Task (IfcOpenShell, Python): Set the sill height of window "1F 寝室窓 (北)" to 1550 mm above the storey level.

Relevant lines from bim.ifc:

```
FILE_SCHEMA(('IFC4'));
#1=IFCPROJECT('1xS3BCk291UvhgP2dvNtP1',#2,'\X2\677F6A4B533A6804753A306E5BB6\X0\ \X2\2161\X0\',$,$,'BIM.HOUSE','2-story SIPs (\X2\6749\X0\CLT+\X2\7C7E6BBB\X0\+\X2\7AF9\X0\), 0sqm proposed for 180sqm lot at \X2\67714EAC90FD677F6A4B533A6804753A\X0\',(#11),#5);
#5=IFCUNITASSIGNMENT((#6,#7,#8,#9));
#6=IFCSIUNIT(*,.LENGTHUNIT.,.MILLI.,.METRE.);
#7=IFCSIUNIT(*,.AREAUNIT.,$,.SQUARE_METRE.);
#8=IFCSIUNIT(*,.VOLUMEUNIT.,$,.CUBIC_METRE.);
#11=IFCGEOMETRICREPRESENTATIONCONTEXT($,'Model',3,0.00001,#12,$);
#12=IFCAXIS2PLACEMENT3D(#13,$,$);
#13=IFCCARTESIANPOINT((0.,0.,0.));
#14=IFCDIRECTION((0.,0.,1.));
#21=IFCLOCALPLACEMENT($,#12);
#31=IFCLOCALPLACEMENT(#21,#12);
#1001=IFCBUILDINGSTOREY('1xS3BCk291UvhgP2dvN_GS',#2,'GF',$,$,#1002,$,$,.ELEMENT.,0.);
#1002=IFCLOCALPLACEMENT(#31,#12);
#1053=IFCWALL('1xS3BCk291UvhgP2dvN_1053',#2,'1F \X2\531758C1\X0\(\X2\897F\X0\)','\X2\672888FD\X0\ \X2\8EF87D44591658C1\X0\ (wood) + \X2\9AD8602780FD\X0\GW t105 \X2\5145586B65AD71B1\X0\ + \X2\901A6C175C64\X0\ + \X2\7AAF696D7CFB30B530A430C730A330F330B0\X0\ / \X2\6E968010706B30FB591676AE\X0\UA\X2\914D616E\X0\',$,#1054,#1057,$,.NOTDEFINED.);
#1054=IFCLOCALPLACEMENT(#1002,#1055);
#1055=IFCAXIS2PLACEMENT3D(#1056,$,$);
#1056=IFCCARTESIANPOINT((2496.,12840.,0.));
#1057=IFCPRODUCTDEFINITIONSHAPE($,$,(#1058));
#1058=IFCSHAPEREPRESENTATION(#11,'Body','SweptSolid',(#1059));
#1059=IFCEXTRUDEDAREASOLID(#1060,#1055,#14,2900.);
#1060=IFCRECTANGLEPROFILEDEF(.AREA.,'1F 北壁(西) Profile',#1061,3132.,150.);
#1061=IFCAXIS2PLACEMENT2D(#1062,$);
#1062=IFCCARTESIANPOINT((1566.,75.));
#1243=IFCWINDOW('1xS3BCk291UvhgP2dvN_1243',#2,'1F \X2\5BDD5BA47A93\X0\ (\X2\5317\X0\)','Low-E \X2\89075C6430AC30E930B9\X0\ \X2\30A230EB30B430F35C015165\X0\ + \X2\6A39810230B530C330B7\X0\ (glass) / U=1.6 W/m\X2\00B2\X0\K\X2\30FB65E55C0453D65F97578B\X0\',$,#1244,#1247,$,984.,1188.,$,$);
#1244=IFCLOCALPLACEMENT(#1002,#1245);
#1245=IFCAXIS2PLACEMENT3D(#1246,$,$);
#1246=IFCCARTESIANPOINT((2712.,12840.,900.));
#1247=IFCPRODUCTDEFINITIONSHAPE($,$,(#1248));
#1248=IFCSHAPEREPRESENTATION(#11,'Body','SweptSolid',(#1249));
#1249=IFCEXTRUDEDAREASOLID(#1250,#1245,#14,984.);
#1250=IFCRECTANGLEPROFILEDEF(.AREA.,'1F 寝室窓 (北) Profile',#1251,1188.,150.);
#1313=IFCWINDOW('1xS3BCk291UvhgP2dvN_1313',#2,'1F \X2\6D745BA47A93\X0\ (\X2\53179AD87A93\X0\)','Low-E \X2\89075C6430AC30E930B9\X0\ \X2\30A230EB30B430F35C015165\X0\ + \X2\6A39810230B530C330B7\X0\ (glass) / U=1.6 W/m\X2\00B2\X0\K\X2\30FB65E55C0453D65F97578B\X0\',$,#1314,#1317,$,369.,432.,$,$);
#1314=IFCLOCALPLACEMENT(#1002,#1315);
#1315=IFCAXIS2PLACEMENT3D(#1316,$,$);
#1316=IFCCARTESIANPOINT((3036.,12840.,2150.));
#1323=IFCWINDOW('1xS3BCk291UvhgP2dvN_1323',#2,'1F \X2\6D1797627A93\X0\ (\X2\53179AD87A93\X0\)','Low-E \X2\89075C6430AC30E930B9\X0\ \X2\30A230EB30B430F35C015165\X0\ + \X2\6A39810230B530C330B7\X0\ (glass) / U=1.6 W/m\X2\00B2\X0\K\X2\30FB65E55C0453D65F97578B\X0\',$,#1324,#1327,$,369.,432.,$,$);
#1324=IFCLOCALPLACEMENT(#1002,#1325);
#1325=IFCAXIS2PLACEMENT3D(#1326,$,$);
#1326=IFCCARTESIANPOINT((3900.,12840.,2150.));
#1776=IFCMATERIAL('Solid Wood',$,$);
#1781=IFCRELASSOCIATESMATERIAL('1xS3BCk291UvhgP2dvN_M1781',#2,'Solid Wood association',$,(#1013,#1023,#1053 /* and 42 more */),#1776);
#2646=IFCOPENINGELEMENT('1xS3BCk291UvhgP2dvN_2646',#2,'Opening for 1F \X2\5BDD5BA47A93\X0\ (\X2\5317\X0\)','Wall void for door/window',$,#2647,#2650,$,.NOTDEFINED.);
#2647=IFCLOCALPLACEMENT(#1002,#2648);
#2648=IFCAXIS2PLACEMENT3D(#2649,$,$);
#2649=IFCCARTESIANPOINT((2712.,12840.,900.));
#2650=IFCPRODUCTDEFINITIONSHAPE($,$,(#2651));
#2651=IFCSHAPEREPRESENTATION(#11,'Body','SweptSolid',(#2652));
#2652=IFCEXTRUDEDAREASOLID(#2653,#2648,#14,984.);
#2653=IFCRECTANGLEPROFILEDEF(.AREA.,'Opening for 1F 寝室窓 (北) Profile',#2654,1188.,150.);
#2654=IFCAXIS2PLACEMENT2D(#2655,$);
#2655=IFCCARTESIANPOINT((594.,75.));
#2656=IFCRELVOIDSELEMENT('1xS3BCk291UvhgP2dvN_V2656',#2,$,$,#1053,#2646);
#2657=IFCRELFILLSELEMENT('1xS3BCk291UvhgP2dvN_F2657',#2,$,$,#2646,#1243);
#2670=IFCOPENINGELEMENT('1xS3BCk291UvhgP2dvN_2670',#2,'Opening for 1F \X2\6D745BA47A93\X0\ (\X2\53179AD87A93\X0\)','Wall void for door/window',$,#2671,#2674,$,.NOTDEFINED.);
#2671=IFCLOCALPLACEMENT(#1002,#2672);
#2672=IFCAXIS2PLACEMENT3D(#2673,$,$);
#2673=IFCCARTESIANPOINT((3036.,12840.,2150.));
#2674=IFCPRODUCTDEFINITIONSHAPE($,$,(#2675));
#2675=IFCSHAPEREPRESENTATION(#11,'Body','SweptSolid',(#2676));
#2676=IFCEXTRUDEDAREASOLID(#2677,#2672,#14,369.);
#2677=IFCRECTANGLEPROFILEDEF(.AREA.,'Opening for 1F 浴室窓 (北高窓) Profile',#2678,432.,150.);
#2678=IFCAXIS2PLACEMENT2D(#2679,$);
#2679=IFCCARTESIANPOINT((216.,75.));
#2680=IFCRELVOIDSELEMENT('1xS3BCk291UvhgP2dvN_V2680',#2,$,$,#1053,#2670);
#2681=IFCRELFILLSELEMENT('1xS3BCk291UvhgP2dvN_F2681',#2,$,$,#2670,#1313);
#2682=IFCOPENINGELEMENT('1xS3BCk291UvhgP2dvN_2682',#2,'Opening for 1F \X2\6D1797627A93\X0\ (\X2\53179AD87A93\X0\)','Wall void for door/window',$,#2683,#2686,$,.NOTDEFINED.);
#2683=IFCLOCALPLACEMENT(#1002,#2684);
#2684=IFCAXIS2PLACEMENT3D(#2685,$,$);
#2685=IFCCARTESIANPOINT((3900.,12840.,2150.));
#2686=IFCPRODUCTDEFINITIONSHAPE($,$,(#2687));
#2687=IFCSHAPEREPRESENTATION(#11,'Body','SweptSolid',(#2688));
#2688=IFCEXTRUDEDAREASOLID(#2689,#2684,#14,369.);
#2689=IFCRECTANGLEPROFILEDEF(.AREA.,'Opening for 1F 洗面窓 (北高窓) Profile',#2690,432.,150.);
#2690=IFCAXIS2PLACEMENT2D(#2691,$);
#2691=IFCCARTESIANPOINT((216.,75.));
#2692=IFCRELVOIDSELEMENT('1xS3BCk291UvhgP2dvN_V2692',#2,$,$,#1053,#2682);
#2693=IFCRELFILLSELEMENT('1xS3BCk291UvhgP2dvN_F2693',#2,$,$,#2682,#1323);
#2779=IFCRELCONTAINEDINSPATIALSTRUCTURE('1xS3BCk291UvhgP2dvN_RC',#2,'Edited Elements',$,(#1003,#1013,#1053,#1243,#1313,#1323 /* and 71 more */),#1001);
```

```python
import numpy as np
import ifcopenshell
import ifcopenshell.api.geometry
import ifcopenshell.geom
import ifcopenshell.util.element
import ifcopenshell.util.placement
import ifcopenshell.util.shape
import ifcopenshell.util.unit

model = ifcopenshell.open("bim.ifc")
unit_scale = ifcopenshell.util.unit.calculate_unit_scale(model)

window = model.by_id(1243)
opening = window.FillsVoids[0].RelatingOpeningElement
storey = ifcopenshell.util.element.get_container(window, ifc_class="IfcBuildingStorey")
level = ifcopenshell.util.placement.get_local_placement(storey.ObjectPlacement)[2, 3]

# The opening's origin need not be at the sill, so measure its lowest point.
shape = ifcopenshell.geom.create_shape(ifcopenshell.geom.settings(), opening)
bottom = ifcopenshell.util.shape.get_shape_bottom_elevation(shape, shape.geometry) / unit_scale
dz = level + 1550.0 - bottom

shift = np.array([0.0, 0.0, dz])
# The window is not placed relative to its opening, so move both.
for product in (opening, window):
    matrix = ifcopenshell.util.placement.get_local_placement(product.ObjectPlacement)
    matrix[:3, 3] += shift
    ifcopenshell.api.geometry.edit_object_placement(model, product=product, matrix=matrix, is_si=False)

print(f"moved by {dz * unit_scale:+.3f} m")

model.write("bim_v2.ifc")
```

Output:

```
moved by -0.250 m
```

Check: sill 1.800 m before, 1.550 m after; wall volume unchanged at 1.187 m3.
